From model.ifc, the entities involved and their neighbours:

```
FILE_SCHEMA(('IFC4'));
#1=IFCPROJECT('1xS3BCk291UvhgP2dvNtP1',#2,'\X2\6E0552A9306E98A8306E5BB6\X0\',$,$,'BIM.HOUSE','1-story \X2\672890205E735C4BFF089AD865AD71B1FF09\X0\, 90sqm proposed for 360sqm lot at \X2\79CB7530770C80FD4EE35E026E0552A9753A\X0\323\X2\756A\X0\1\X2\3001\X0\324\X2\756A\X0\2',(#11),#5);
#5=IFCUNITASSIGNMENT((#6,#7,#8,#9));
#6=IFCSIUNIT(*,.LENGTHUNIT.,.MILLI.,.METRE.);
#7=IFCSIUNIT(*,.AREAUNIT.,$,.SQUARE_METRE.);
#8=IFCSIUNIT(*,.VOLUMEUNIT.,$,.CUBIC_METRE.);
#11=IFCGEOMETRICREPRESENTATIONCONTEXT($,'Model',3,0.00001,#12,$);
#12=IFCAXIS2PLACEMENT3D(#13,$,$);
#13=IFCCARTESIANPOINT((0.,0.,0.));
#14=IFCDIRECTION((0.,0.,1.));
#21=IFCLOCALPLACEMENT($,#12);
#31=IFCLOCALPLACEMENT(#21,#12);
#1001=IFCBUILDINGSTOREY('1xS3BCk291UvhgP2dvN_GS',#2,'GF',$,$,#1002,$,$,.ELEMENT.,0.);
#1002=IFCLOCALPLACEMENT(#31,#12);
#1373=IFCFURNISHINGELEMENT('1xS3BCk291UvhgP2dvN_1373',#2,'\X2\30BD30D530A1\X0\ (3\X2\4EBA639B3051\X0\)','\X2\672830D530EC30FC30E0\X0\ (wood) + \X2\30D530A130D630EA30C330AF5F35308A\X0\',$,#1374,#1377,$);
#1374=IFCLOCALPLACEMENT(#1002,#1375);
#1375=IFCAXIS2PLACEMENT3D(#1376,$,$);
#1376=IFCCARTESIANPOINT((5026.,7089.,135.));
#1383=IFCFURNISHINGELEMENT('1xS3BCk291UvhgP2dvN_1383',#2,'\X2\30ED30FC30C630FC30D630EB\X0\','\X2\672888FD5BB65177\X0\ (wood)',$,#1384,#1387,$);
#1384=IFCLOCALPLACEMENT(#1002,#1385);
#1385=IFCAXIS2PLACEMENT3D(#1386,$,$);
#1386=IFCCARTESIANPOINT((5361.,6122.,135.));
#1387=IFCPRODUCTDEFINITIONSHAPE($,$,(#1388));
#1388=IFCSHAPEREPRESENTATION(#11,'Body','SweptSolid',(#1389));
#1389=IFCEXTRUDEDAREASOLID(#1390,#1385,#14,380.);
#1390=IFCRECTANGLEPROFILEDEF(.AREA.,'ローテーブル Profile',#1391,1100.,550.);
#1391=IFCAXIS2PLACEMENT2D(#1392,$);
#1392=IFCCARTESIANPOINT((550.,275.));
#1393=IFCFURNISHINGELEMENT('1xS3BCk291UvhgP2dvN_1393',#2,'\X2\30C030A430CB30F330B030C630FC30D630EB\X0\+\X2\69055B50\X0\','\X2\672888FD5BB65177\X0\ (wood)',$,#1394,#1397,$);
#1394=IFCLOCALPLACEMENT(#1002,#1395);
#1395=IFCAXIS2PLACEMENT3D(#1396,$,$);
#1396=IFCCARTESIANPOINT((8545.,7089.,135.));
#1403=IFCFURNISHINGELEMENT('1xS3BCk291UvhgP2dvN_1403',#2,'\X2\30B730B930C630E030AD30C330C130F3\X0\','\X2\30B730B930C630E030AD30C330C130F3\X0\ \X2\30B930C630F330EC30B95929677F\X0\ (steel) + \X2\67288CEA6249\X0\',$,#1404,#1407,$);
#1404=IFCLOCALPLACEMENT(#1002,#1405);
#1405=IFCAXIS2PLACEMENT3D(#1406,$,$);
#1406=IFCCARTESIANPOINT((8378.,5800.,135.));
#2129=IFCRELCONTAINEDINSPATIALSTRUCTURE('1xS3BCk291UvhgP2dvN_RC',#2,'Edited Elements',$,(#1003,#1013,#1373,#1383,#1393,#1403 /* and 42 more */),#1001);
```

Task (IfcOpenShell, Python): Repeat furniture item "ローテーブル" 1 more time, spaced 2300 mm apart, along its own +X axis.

```python
import ifcopenshell
import ifcopenshell.api.geometry
import ifcopenshell.api.root
import ifcopenshell.util.element
import ifcopenshell.util.placement
import ifcopenshell.util.unit

model = ifcopenshell.open("model.ifc")
unit_scale = ifcopenshell.util.unit.calculate_unit_scale(model)


def reuse_history(source, copy):
    """copy_class also copies each property set's owner history, people and application; keep the originals."""
    for rel in copy.IsDefinedBy:
        if rel.is_a("IfcRelDefinesByProperties") and (history := rel.RelatingPropertyDefinition.OwnerHistory):
            rel.RelatingPropertyDefinition.OwnerHistory = source.OwnerHistory
            ifcopenshell.util.element.remove_deep2(model, history)


source = model.by_guid("1xS3BCk291UvhgP2dvN_1383")
base = ifcopenshell.util.placement.get_local_placement(source.ObjectPlacement)
step = base[:3, 0] * 2.3 / unit_scale

for i in range(1, 2):
    copy = ifcopenshell.api.root.copy_class(model, product=source)
    copy.Representation = ifcopenshell.util.element.copy_deep(
        model, source.Representation, exclude=["IfcGeometricRepresentationContext", "IfcRepresentationMap"]
    )
    reuse_history(source, copy)
    matrix = base.copy()
    matrix[:3, 3] += i * step
    print("added at", matrix[:3, 3].round(3) + 0.0)
    ifcopenshell.api.geometry.edit_object_placement(model, product=copy, matrix=matrix, is_si=False)

model.write("model-out.ifc")
```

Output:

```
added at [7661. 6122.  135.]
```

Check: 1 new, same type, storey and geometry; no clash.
